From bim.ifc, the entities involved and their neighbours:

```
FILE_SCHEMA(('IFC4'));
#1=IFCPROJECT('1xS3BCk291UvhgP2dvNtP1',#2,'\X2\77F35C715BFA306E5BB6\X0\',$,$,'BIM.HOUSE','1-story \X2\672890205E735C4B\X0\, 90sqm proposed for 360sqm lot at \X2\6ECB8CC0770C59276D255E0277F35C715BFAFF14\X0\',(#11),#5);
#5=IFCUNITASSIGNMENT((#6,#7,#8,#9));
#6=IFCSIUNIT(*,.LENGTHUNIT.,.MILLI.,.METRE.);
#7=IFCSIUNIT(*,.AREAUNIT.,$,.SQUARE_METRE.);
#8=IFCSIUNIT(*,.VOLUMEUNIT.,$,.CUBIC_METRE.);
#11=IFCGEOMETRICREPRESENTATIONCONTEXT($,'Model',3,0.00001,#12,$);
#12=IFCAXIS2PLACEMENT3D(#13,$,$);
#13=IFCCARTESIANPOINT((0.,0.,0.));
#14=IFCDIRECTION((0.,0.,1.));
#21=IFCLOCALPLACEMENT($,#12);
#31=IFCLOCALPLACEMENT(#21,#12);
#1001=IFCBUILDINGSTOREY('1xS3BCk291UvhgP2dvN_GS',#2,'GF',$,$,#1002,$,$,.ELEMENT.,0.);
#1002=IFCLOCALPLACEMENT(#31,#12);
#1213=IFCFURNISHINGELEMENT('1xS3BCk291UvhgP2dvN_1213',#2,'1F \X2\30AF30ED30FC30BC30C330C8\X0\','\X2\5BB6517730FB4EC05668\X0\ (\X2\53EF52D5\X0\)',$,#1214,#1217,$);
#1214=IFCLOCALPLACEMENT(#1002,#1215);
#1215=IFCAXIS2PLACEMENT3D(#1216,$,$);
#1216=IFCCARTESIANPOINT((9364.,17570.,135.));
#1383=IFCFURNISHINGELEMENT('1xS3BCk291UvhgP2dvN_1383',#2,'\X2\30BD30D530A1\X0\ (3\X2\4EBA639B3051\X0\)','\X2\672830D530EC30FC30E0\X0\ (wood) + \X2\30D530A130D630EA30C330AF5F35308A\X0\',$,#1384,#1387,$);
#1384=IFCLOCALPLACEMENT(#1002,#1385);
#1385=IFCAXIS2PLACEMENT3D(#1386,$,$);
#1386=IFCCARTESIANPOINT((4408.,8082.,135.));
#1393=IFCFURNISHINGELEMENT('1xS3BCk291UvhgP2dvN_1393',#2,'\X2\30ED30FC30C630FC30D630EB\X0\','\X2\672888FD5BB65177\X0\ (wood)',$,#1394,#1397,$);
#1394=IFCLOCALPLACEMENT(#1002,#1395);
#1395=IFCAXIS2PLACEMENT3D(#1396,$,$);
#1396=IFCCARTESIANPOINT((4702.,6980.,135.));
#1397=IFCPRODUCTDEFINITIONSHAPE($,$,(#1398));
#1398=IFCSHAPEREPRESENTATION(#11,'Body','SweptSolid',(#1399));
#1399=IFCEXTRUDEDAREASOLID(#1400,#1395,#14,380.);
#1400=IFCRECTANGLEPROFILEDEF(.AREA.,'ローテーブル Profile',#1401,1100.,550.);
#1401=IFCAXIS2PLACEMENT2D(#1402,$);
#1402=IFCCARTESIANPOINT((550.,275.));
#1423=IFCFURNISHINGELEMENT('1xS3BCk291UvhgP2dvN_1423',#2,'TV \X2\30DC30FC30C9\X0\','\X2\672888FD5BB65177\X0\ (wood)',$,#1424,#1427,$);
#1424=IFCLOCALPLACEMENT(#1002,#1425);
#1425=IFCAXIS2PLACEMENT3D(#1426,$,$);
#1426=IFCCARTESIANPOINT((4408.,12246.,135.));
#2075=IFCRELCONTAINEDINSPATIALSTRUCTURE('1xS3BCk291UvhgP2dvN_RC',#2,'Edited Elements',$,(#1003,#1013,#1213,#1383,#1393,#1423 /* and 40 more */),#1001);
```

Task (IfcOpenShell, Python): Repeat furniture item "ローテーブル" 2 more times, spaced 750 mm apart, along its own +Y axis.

```python
import ifcopenshell
import ifcopenshell.api.geometry
import ifcopenshell.api.root
import ifcopenshell.util.element
import ifcopenshell.util.placement
import ifcopenshell.util.unit

model = ifcopenshell.open("bim.ifc")
unit_scale = ifcopenshell.util.unit.calculate_unit_scale(model)


def reuse_history(source, copy):
    """copy_class also copies each property set's owner history, people and application; keep the originals."""
    for rel in copy.IsDefinedBy:
        if rel.is_a("IfcRelDefinesByProperties") and (history := rel.RelatingPropertyDefinition.OwnerHistory):
            rel.RelatingPropertyDefinition.OwnerHistory = source.OwnerHistory
            ifcopenshell.util.element.remove_deep2(model, history)


source = model.by_guid("1xS3BCk291UvhgP2dvN_1393")
base = ifcopenshell.util.placement.get_local_placement(source.ObjectPlacement)
step = base[:3, 1] * 0.75 / unit_scale

for i in range(1, 3):
    copy = ifcopenshell.api.root.copy_class(model, product=source)
    copy.Representation = ifcopenshell.util.element.copy_deep(
        model, source.Representation, exclude=["IfcGeometricRepresentationContext", "IfcRepresentationMap"]
    )
    reuse_history(source, copy)
    matrix = base.copy()
    matrix[:3, 3] += i * step
    print("added at", matrix[:3, 3].round(3) + 0.0)
    ifcopenshell.api.geometry.edit_object_placement(model, product=copy, matrix=matrix, is_si=False)

model.write("bim-out.ifc")
```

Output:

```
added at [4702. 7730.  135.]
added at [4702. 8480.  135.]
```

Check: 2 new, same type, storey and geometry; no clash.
